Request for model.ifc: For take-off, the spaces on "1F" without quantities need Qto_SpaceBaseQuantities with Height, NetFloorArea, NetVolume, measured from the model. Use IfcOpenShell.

First a look at what the model holds.

```python
import ifcopenshell
import ifcopenshell.util.element
import ifcopenshell.util.unit

model = ifcopenshell.open("model.ifc")
print(model.schema)
for unit_type in ("LENGTHUNIT", "AREAUNIT", "VOLUMEUNIT"):
    print(unit_type, ifcopenshell.util.unit.calculate_unit_scale(model, unit_type))
storey = next(s for s in model.by_type("IfcBuildingStorey") if s.Name == "1F")
spaces = [e for e in ifcopenshell.util.element.get_decomposition(storey) if e.is_a("IfcSpace")]
for e in sorted(spaces, key=lambda e: e.id()):
    print(e.id(), e.is_a(), e.Name, list(ifcopenshell.util.element.get_psets(e, qtos_only=True)), sep=" | ")
```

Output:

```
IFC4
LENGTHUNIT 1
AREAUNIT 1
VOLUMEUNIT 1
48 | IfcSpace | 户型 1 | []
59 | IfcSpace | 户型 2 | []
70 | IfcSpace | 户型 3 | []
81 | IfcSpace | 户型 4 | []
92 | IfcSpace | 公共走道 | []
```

```python
import ifcopenshell
import ifcopenshell.api.pset
import ifcopenshell.geom
import ifcopenshell.util.element
import ifcopenshell.util.shape
import ifcopenshell.util.unit

model = ifcopenshell.open("model.ifc")
unit_scale = ifcopenshell.util.unit.calculate_unit_scale(model)
area_scale = ifcopenshell.util.unit.calculate_unit_scale(model, "AREAUNIT")
volume_scale = ifcopenshell.util.unit.calculate_unit_scale(model, "VOLUMEUNIT")
settings = ifcopenshell.geom.settings()

storey = next(s for s in model.by_type("IfcBuildingStorey") if s.Name == "1F")
spaces = [e for e in ifcopenshell.util.element.get_decomposition(storey) if e.is_a("IfcSpace")]

for e in sorted(spaces, key=lambda e: e.id()):
    if ifcopenshell.util.element.get_psets(e, qtos_only=True, should_inherit=False):
        continue
    # Geometry comes back in metres, in the element's own axes.
    shape = ifcopenshell.geom.create_shape(settings, e)
    values = {
        "Height": ifcopenshell.util.shape.get_z(shape.geometry) / unit_scale,
        "NetFloorArea": ifcopenshell.util.shape.get_footprint_area(shape.geometry) / area_scale,
        "NetVolume": ifcopenshell.util.shape.get_volume(shape.geometry) / volume_scale,
    }
    qto = ifcopenshell.api.pset.add_qto(model, product=e, name="Qto_SpaceBaseQuantities")
    ifcopenshell.api.pset.edit_qto(model, qto=qto, properties=values)
    print(e.id(), {k: round(v, 3) for k, v in values.items()})

model.write("model_updated.ifc")
```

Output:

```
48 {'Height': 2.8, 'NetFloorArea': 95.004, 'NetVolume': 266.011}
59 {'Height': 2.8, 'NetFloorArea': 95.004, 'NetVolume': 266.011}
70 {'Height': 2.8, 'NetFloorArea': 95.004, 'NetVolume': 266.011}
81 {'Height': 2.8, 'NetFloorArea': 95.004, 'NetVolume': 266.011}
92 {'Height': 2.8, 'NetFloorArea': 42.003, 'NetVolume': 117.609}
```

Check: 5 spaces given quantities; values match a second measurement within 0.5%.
